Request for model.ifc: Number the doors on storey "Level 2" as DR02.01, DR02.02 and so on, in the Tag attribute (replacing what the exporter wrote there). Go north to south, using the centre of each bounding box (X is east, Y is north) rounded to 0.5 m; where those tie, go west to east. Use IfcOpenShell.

First a look at what the model holds.

```python
import ifcopenshell
import ifcopenshell.util.element
import ifcopenshell.util.placement

model = ifcopenshell.open("model.ifc")
print(model.schema)
storey = next(s for s in model.by_type("IfcBuildingStorey") if s.Name == "Level 2")
doors = [e for e in ifcopenshell.util.element.get_decomposition(storey) if e.is_a("IfcDoor")]
for e in sorted(doors, key=lambda e: e.id()):
    origin = ifcopenshell.util.placement.get_local_placement(e.ObjectPlacement)[:3, 3]
    print(e.id(), e.Tag, e.Name, origin.round(2) + 0.0, sep=" | ")
```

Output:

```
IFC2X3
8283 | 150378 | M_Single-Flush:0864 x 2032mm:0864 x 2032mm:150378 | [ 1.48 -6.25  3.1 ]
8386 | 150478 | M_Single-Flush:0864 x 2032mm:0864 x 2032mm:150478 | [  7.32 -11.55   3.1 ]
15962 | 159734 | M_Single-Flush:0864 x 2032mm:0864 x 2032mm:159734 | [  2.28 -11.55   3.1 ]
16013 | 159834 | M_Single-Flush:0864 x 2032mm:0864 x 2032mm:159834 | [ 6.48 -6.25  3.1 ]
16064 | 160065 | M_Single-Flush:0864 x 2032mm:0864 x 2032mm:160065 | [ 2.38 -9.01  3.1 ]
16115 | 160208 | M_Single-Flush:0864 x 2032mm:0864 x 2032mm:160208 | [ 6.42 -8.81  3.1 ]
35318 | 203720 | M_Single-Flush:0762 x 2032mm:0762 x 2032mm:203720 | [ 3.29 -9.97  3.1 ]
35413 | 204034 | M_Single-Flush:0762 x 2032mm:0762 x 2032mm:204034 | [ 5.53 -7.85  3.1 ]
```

```python
import ifcopenshell
import ifcopenshell.geom
import ifcopenshell.util.element
import ifcopenshell.util.shape

model = ifcopenshell.open("model.ifc")
settings = ifcopenshell.geom.settings()
settings.set("use-world-coords", True)


def centre(element):
    shape = ifcopenshell.geom.create_shape(settings, element)
    return ifcopenshell.util.shape.get_bbox_centroid(shape.geometry)


storey = next(s for s in model.by_type("IfcBuildingStorey") if s.Name == "Level 2")
doors = [e for e in ifcopenshell.util.element.get_decomposition(storey) if e.is_a("IfcDoor")]

# Insertion points can sit at a corner or the storey origin, so sort by the geometry (in metres).
centres = {e: centre(e) for e in doors}
doors.sort(key=lambda e: (-round(centres[e][1] / 0.5), centres[e][0]))

for i, e in enumerate(doors, start=1):
    number = f"DR02.{i:02d}"
    e.Tag = number
    print(e.id(), number)

model.write("model-out.ifc")
```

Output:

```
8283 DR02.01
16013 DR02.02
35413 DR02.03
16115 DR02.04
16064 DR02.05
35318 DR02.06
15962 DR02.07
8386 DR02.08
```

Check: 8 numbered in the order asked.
